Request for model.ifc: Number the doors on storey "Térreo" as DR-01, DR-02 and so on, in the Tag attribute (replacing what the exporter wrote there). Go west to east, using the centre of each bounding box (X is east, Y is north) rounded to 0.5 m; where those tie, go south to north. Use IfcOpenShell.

First a look at what the model holds.

```python
import ifcopenshell
import ifcopenshell.util.element
import ifcopenshell.util.placement

model = ifcopenshell.open("model.ifc")
print(model.schema)
storey = next(s for s in model.by_type("IfcBuildingStorey") if s.Name == "Térreo")
doors = [e for e in ifcopenshell.util.element.get_decomposition(storey) if e.is_a("IfcDoor")]
for e in sorted(doors, key=lambda e: e.id()):
    origin = ifcopenshell.util.placement.get_local_placement(e.ObjectPlacement)[:3, 3]
    print(e.id(), e.Tag, e.Name, origin.round(2) + 0.0, sep=" | ")
```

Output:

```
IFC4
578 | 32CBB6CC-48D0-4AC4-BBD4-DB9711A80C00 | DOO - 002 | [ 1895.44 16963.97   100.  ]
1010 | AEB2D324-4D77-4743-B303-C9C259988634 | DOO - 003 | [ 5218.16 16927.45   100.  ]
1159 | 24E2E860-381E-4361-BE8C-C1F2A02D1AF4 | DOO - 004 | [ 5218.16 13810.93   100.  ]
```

```python
import ifcopenshell
import ifcopenshell.geom
import ifcopenshell.util.element
import ifcopenshell.util.shape

model = ifcopenshell.open("model.ifc")
settings = ifcopenshell.geom.settings()
settings.set("use-world-coords", True)


def centre(element):
    shape = ifcopenshell.geom.create_shape(settings, element)
    return ifcopenshell.util.shape.get_bbox_centroid(shape.geometry)


storey = next(s for s in model.by_type("IfcBuildingStorey") if s.Name == "Térreo")
doors = [e for e in ifcopenshell.util.element.get_decomposition(storey) if e.is_a("IfcDoor")]

# Insertion points can sit at a corner or the storey origin, so sort by the geometry (in metres).
centres = {e: centre(e) for e in doors}
doors.sort(key=lambda e: (round(centres[e][0] / 0.5), centres[e][1]))

for i, e in enumerate(doors, start=1):
    number = f"DR-{i:02d}"
    e.Tag = number
    print(e.id(), number)

model.write("model_updated.ifc")
```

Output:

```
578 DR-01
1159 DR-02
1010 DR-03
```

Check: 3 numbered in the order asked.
